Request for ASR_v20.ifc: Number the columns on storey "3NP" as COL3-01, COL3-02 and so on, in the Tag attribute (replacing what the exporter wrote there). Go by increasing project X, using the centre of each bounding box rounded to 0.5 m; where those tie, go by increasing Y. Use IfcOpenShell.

First a look at what the model holds.

```python
import ifcopenshell
import ifcopenshell.util.element
import ifcopenshell.util.placement

model = ifcopenshell.open("ASR_v20.ifc")
print(model.schema)
storey = next(s for s in model.by_type("IfcBuildingStorey") if s.Name == "3NP")
columns = [e for e in ifcopenshell.util.element.get_decomposition(storey) if e.is_a("IfcColumn")]
for e in sorted(columns, key=lambda e: e.id()):
    origin = ifcopenshell.util.placement.get_local_placement(e.ObjectPlacement)[:3, 3]
    print(e.id(), e.Tag, e.Name, origin.round(2) + 0.0, sep=" | ")
```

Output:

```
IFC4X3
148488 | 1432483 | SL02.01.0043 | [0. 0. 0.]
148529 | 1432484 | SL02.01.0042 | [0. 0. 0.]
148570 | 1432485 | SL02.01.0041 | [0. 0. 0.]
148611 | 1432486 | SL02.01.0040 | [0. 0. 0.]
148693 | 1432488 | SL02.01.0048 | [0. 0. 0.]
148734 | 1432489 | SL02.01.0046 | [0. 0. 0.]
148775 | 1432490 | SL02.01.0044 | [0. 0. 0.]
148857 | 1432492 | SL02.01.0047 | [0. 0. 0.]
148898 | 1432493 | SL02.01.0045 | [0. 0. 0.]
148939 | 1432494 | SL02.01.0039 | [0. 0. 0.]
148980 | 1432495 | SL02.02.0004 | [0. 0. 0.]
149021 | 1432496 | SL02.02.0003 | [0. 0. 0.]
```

```python
import ifcopenshell
import ifcopenshell.geom
import ifcopenshell.util.element
import ifcopenshell.util.shape

model = ifcopenshell.open("ASR_v20.ifc")
settings = ifcopenshell.geom.settings()
settings.set("use-world-coords", True)


def centre(element):
    shape = ifcopenshell.geom.create_shape(settings, element)
    return ifcopenshell.util.shape.get_bbox_centroid(shape.geometry)


storey = next(s for s in model.by_type("IfcBuildingStorey") if s.Name == "3NP")
columns = [e for e in ifcopenshell.util.element.get_decomposition(storey) if e.is_a("IfcColumn")]

# Insertion points can sit at a corner or the storey origin, so sort by the geometry (in metres).
centres = {e: centre(e) for e in columns}
columns.sort(key=lambda e: (round(centres[e][0] / 0.5), centres[e][1]))

for i, e in enumerate(columns, start=1):
    number = f"COL3-{i:02d}"
    e.Tag = number
    print(e.id(), number)

model.write("ASR_v20_v2.ifc")
```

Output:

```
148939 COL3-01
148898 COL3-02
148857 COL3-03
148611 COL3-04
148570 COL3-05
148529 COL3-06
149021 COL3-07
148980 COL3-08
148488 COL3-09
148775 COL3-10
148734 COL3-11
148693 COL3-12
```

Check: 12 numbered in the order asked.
